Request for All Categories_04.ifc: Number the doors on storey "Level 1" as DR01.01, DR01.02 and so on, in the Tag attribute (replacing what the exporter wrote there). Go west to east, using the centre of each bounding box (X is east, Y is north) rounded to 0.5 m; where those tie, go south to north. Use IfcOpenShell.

First a look at what the model holds.

```python
import ifcopenshell
import ifcopenshell.util.element
import ifcopenshell.util.placement

model = ifcopenshell.open("All Categories_04.ifc")
print(model.schema)
storey = next(s for s in model.by_type("IfcBuildingStorey") if s.Name == "Level 1")
doors = [e for e in ifcopenshell.util.element.get_decomposition(storey) if e.is_a("IfcDoor")]
for e in sorted(doors, key=lambda e: e.id()):
    origin = ifcopenshell.util.placement.get_local_placement(e.ObjectPlacement)[:3, 3]
    print(e.id(), e.Tag, e.Name, origin.round(2) + 0.0, sep=" | ")
```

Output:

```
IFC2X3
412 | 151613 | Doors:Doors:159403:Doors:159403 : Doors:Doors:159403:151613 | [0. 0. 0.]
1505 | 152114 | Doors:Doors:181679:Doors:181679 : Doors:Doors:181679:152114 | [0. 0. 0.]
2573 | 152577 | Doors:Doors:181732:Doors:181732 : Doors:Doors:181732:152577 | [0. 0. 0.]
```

```python
import ifcopenshell
import ifcopenshell.geom
import ifcopenshell.util.element
import ifcopenshell.util.shape

model = ifcopenshell.open("All Categories_04.ifc")
settings = ifcopenshell.geom.settings()
settings.set("use-world-coords", True)


def centre(element):
    shape = ifcopenshell.geom.create_shape(settings, element)
    return ifcopenshell.util.shape.get_bbox_centroid(shape.geometry)


storey = next(s for s in model.by_type("IfcBuildingStorey") if s.Name == "Level 1")
doors = [e for e in ifcopenshell.util.element.get_decomposition(storey) if e.is_a("IfcDoor")]

# Insertion points can sit at a corner or the storey origin, so sort by the geometry (in metres).
centres = {e: centre(e) for e in doors}
doors.sort(key=lambda e: (round(centres[e][0] / 0.5), centres[e][1]))

for i, e in enumerate(doors, start=1):
    number = f"DR01.{i:02d}"
    e.Tag = number
    print(e.id(), number)

model.write("All Categories_04_updated.ifc")
```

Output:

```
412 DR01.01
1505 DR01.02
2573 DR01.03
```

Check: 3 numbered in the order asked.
